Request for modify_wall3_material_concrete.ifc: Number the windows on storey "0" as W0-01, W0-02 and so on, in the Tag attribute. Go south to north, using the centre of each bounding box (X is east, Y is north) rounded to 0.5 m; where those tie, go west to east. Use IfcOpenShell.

First a look at what the model holds.

```python
import ifcopenshell
import ifcopenshell.util.element
import ifcopenshell.util.placement

model = ifcopenshell.open("modify_wall3_material_concrete.ifc")
print(model.schema)
storey = next(s for s in model.by_type("IfcBuildingStorey") if s.Name == "0")
windows = [e for e in ifcopenshell.util.element.get_decomposition(storey) if e.is_a("IfcWindow")]
for e in sorted(windows, key=lambda e: e.id()):
    origin = ifcopenshell.util.placement.get_local_placement(e.ObjectPlacement)[:3, 3]
    print(e.id(), e.Tag, e.Name, origin.round(2) + 0.0, sep=" | ")
```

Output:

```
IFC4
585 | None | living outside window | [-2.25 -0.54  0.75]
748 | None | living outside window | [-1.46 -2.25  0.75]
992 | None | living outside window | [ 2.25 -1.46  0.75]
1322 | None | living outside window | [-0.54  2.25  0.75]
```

```python
import ifcopenshell
import ifcopenshell.geom
import ifcopenshell.util.element
import ifcopenshell.util.shape

model = ifcopenshell.open("modify_wall3_material_concrete.ifc")
settings = ifcopenshell.geom.settings()
settings.set("use-world-coords", True)


def centre(element):
    shape = ifcopenshell.geom.create_shape(settings, element)
    return ifcopenshell.util.shape.get_bbox_centroid(shape.geometry)


storey = next(s for s in model.by_type("IfcBuildingStorey") if s.Name == "0")
windows = [e for e in ifcopenshell.util.element.get_decomposition(storey) if e.is_a("IfcWindow")]

# Insertion points can sit at a corner or the storey origin, so sort by the geometry (in metres).
centres = {e: centre(e) for e in windows}
windows.sort(key=lambda e: (round(centres[e][1] / 0.5), centres[e][0]))

for i, e in enumerate(windows, start=1):
    number = f"W0-{i:02d}"
    e.Tag = number
    print(e.id(), number)

model.write("modify_wall3_material_concrete_rev.ifc")
```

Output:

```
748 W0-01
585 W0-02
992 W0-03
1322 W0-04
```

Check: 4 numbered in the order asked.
